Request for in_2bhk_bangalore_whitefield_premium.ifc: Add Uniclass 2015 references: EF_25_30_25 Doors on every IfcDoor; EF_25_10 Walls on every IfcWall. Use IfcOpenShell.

First a look at what the model holds.

```python
import ifcopenshell

model = ifcopenshell.open("in_2bhk_bangalore_whitefield_premium.ifc")
print(model.schema)
print("classifications:", [c.Name for c in model.by_type("IfcClassification")])
for ifc_class in ("IfcDoor", "IfcRoof", "IfcStair", "IfcWall", "IfcWindow"):
    print(ifc_class, len(model.by_type(ifc_class)))
```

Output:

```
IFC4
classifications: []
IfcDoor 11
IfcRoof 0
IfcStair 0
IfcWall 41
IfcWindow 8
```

```python
import ifcopenshell
import ifcopenshell.api.classification

model = ifcopenshell.open("in_2bhk_bangalore_whitefield_premium.ifc")

system = ifcopenshell.api.classification.add_classification(model, classification="Uniclass 2015")

codes = {
    "IfcDoor": ("EF_25_30_25", "Doors"),
    "IfcWall": ("EF_25_10", "Walls"),
}
for ifc_class, (code, name) in codes.items():
    products = model.by_type(ifc_class)
    ifcopenshell.api.classification.add_reference(
        model, products=products, classification=system, identification=code, name=name
    )
    print(code, len(products))

model.write("in_2bhk_bangalore_whitefield_premium_edited.ifc")
```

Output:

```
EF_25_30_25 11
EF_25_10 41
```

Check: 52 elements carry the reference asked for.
